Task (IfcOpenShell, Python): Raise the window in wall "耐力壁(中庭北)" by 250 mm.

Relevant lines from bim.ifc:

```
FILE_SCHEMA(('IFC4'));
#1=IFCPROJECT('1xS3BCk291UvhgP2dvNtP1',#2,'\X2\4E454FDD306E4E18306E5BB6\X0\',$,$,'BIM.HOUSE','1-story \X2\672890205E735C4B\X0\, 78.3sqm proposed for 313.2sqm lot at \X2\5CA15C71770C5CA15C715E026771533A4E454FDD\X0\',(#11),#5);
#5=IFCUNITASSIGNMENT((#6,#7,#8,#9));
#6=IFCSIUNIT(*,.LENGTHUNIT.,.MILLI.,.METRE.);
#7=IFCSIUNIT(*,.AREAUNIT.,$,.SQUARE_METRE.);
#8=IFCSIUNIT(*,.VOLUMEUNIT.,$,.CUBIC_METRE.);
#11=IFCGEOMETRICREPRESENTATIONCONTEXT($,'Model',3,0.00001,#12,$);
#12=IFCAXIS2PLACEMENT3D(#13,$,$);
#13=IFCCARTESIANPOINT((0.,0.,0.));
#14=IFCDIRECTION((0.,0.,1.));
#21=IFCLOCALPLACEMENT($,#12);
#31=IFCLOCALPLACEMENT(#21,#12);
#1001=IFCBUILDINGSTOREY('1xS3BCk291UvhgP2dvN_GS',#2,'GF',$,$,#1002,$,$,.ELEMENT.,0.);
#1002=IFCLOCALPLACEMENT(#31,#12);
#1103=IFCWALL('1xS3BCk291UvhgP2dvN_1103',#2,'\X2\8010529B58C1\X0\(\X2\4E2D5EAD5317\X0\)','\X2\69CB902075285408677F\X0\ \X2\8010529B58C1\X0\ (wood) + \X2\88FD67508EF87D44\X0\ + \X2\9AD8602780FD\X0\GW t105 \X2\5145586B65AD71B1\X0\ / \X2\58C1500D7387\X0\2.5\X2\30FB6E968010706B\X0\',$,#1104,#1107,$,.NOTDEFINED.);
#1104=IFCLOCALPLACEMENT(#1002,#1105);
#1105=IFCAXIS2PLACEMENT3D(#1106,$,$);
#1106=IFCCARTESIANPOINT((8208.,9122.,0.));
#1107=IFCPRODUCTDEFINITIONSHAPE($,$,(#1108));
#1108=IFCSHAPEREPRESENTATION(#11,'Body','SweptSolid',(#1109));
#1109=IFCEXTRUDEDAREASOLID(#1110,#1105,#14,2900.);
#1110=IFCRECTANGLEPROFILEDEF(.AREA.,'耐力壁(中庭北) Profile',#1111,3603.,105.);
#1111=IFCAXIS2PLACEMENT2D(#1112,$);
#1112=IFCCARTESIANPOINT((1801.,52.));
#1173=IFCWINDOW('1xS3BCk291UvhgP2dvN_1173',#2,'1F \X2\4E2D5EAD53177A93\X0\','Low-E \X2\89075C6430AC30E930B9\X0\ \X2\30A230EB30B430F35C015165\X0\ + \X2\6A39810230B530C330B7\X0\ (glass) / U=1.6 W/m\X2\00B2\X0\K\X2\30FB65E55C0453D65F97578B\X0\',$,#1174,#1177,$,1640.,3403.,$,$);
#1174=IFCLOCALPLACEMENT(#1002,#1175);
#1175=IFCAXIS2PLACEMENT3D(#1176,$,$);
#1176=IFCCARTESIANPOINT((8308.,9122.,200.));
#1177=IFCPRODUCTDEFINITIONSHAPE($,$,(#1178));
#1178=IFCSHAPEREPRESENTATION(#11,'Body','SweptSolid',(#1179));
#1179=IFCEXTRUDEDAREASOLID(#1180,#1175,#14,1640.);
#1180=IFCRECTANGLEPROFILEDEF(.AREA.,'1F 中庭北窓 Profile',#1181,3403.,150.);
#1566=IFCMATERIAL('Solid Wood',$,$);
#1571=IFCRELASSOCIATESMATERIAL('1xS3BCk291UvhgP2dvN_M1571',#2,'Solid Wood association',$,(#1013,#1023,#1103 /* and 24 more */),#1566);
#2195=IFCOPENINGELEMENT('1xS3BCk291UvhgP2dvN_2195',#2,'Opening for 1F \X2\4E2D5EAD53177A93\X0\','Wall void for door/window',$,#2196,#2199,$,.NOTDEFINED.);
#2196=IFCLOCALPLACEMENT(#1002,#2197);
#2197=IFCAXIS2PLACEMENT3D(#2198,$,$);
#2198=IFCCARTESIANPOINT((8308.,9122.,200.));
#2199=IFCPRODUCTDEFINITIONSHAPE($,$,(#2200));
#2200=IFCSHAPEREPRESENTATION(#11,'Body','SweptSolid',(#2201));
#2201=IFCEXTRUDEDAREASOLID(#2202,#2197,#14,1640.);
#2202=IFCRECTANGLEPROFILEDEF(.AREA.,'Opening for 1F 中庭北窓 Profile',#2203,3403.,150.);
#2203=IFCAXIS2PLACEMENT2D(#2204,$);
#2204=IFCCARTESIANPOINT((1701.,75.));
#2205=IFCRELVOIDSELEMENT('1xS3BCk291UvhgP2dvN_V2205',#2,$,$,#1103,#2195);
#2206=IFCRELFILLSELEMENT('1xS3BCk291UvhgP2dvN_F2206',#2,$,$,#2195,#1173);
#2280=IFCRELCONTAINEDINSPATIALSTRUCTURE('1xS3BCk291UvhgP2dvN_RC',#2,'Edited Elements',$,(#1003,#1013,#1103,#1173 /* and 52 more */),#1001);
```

```python
import numpy as np
import ifcopenshell
import ifcopenshell.api.geometry
import ifcopenshell.util.placement
import ifcopenshell.util.unit

model = ifcopenshell.open("bim.ifc")
unit_scale = ifcopenshell.util.unit.calculate_unit_scale(model)

window = model.by_guid("1xS3BCk291UvhgP2dvN_1173")
opening = window.FillsVoids[0].RelatingOpeningElement
dz = 0.25 / unit_scale

shift = np.array([0.0, 0.0, dz])
# The window is not placed relative to its opening, so move both.
for product in (opening, window):
    matrix = ifcopenshell.util.placement.get_local_placement(product.ObjectPlacement)
    matrix[:3, 3] += shift
    ifcopenshell.api.geometry.edit_object_placement(model, product=product, matrix=matrix, is_si=False)

print(f"moved by {dz * unit_scale:+.3f} m")

model.write("bim-out.ifc")
```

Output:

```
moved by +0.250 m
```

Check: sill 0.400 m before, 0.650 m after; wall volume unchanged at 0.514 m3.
